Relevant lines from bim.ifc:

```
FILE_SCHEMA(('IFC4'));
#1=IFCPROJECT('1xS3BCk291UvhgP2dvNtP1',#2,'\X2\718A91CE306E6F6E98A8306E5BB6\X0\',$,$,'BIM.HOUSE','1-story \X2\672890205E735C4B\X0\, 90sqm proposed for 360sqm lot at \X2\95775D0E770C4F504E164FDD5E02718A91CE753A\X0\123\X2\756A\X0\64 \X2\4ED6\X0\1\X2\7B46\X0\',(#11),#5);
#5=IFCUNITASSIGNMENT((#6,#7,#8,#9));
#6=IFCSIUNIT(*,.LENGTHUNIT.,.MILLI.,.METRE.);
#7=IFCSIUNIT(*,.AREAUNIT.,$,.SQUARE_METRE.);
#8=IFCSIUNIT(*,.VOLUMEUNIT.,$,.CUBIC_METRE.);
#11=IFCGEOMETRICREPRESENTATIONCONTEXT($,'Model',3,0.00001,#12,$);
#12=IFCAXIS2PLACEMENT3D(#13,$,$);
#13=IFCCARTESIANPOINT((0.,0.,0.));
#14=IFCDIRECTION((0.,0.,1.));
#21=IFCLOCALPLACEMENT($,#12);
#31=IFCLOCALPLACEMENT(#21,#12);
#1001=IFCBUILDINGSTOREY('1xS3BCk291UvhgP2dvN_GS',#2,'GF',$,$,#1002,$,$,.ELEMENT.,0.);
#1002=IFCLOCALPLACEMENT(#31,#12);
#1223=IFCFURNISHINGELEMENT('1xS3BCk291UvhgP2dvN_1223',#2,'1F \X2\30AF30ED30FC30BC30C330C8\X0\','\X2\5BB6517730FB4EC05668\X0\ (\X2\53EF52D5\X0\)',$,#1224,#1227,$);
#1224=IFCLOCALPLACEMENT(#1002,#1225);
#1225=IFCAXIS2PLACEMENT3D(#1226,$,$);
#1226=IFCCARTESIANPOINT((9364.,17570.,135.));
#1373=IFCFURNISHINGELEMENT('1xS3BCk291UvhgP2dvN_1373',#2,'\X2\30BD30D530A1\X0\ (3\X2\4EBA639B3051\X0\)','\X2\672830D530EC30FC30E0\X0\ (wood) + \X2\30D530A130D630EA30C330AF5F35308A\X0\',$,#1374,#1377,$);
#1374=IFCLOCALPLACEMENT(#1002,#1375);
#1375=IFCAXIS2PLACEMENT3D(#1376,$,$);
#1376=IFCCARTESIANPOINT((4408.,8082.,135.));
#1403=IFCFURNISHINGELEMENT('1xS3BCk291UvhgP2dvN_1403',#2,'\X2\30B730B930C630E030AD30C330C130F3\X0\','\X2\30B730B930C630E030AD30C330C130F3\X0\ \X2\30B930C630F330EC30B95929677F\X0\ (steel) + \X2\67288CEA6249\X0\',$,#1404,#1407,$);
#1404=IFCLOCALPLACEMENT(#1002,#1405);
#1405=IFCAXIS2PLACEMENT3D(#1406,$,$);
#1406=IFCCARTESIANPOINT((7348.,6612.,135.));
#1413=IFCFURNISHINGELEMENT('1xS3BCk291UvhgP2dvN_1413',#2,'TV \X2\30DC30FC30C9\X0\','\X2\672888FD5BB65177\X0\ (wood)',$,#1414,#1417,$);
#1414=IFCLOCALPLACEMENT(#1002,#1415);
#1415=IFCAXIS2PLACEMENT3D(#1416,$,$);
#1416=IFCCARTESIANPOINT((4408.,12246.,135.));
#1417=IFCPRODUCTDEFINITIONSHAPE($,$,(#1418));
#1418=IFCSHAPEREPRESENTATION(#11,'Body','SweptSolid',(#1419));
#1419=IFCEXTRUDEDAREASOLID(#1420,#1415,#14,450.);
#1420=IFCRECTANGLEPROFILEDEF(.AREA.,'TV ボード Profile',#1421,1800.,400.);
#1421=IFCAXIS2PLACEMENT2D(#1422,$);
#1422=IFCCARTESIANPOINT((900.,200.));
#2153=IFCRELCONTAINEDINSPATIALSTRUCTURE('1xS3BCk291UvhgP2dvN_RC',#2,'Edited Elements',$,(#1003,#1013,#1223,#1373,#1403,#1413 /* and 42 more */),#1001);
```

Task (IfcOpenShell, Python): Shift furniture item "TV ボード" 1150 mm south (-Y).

```python
import ifcopenshell
import ifcopenshell.api.geometry
import ifcopenshell.util.placement

model = ifcopenshell.open("bim.ifc")

item = model.by_id(1413)
matrix = ifcopenshell.util.placement.get_local_placement(item.ObjectPlacement)
matrix[1, 3] -= 1150.0
ifcopenshell.api.geometry.edit_object_placement(model, product=item, matrix=matrix, is_si=False)

print(ifcopenshell.util.placement.get_local_placement(item.ObjectPlacement).round(3) + 0.0)

model.write("bim_v2.ifc")
```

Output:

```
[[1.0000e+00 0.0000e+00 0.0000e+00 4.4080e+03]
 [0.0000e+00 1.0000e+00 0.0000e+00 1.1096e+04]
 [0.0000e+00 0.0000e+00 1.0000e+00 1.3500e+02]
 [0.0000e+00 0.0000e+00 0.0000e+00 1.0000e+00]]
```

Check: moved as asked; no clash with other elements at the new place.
